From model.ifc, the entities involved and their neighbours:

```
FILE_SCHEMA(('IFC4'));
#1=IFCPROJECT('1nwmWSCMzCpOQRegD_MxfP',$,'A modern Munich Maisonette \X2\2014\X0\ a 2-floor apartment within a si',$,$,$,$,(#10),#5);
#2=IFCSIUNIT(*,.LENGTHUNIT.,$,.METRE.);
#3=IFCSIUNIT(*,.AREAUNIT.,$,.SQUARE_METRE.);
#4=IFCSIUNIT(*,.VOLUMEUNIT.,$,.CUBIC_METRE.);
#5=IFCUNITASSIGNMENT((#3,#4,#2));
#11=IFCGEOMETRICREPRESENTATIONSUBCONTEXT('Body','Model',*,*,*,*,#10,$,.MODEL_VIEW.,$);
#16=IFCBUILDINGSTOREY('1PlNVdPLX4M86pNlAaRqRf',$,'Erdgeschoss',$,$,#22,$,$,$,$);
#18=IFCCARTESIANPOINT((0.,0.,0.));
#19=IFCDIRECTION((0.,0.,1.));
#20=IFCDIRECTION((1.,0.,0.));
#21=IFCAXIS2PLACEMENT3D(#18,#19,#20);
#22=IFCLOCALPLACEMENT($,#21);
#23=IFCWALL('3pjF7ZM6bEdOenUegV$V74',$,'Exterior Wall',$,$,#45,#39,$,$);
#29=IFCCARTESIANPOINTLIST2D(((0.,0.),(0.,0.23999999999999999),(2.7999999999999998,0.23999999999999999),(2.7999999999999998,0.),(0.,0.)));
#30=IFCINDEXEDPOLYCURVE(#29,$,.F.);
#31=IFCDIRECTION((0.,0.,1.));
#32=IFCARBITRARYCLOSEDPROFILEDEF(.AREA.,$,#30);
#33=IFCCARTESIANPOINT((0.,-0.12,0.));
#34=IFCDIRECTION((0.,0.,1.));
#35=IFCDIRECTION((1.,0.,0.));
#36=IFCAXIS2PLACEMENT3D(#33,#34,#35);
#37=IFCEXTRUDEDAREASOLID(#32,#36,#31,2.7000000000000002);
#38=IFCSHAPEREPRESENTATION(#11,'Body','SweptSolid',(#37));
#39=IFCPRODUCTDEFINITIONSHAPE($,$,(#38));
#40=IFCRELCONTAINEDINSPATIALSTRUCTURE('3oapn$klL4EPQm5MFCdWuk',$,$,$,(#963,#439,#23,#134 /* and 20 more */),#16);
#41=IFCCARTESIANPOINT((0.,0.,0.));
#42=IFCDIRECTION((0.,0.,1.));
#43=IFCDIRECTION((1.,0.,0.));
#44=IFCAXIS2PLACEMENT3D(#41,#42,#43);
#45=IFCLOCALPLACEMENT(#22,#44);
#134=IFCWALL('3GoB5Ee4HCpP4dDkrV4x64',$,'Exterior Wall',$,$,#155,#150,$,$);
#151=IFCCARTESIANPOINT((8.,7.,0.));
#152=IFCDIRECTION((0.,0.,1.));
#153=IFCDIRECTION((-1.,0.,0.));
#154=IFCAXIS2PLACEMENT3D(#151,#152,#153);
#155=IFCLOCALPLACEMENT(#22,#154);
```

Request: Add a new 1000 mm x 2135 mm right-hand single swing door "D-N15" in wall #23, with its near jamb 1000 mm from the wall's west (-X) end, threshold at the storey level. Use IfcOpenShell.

```python
import numpy as np
import ifcopenshell
import ifcopenshell.api.feature
import ifcopenshell.api.geometry
import ifcopenshell.api.root
import ifcopenshell.api.spatial
import ifcopenshell.geom
import ifcopenshell.util.element
import ifcopenshell.util.placement
import ifcopenshell.util.representation
import ifcopenshell.util.shape
import ifcopenshell.util.unit

model = ifcopenshell.open("model.ifc")
unit_scale = ifcopenshell.util.unit.calculate_unit_scale(model)
settings = ifcopenshell.geom.settings()


def volume(element):
    """Net volume in cubic metres, openings subtracted."""
    shape = ifcopenshell.geom.create_shape(settings, element)
    return ifcopenshell.util.shape.get_volume(shape.geometry)


wall = model.by_guid("3pjF7ZM6bEdOenUegV$V74")
storey = ifcopenshell.util.element.get_container(wall, ifc_class="IfcBuildingStorey")
context = ifcopenshell.util.representation.get_context(model, "Model", "Body", "MODEL_VIEW")
before = volume(wall)

width, height, from_end, sill = 1, 2.135, 1, 0.0  # metres

# The wall runs along its own X axis, and the end named is its -X end.
wall_shape = ifcopenshell.geom.create_shape(settings, wall)
x, y, z = ifcopenshell.util.shape.get_vertices(wall_shape.geometry).T
start = x.min() + from_end
face, thickness = float(y.min()), float(y.max() - y.min())
wall_matrix = ifcopenshell.util.placement.get_local_placement(wall.ObjectPlacement)
level = ifcopenshell.util.placement.get_local_placement(storey.ObjectPlacement)[2, 3]


def in_wall(x, y):
    """Placement at x, y metres in the wall's axes, at sill height."""
    matrix = wall_matrix.copy()
    matrix[:, 3] = wall_matrix @ np.array([x / unit_scale, y / unit_scale, 0.0, 1.0])
    matrix[2, 3] = level + sill / unit_scale
    return matrix


# Opening: a box that overshoots both wall faces by 50 mm.
opening = ifcopenshell.api.root.create_entity(model, ifc_class="IfcOpeningElement", predefined_type="OPENING")
box = ifcopenshell.api.geometry.add_wall_representation(
    model, context=context, length=width, height=height, thickness=thickness + 0.1
)
ifcopenshell.api.geometry.assign_representation(model, product=opening, representation=box)
ifcopenshell.api.geometry.edit_object_placement(model, product=opening, matrix=in_wall(start, face - 0.05), is_si=False)
ifcopenshell.api.feature.add_feature(model, feature=opening, element=wall)

door = ifcopenshell.api.root.create_entity(model, ifc_class="IfcDoor", name="D-N15", predefined_type="DOOR")
door.OverallWidth, door.OverallHeight = width / unit_scale, height / unit_scale
door.OperationType = "SINGLE_SWING_RIGHT"
body = ifcopenshell.api.geometry.add_door_representation(
    model,
    context=context,
    overall_width=door.OverallWidth,
    overall_height=door.OverallHeight,
    operation_type="SINGLE_SWING_RIGHT",
    lining_properties={"LiningDepth": thickness / unit_scale, "ThresholdDepth": thickness / unit_scale},
)
ifcopenshell.api.geometry.assign_representation(model, product=door, representation=body)
ifcopenshell.api.spatial.assign_container(model, products=[door], relating_structure=storey)
ifcopenshell.api.feature.add_filling(model, opening=opening, element=door)

# The lining spans the wall, so the door starts at the wall face.
ifcopenshell.api.geometry.edit_object_placement(model, product=door, matrix=in_wall(start, face), is_si=False)

after = volume(wall)

print(f"wall volume {before:.3f} -> {after:.3f} m3")

model.write("model-out.ifc")
```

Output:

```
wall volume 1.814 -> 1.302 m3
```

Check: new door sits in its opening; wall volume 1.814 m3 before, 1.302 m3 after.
